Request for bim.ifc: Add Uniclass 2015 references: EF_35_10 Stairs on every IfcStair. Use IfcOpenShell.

First a look at what the model holds.

```python
import ifcopenshell

model = ifcopenshell.open("bim.ifc")
print(model.schema)
print("classifications:", [c.Name for c in model.by_type("IfcClassification")])
for ifc_class in ("IfcDoor", "IfcRoof", "IfcStair", "IfcWall", "IfcWindow"):
    print(ifc_class, len(model.by_type(ifc_class)))
```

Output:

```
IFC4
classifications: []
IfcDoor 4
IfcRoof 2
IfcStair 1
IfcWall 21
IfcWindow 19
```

```python
import ifcopenshell
import ifcopenshell.api.classification

model = ifcopenshell.open("bim.ifc")

system = ifcopenshell.api.classification.add_classification(model, classification="Uniclass 2015")

codes = {
    "IfcStair": ("EF_35_10", "Stairs"),
}
for ifc_class, (code, name) in codes.items():
    products = model.by_type(ifc_class)
    ifcopenshell.api.classification.add_reference(
        model, products=products, classification=system, identification=code, name=name
    )
    print(code, len(products))

model.write("bim_rev.ifc")
```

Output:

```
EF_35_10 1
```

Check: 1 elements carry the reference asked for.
